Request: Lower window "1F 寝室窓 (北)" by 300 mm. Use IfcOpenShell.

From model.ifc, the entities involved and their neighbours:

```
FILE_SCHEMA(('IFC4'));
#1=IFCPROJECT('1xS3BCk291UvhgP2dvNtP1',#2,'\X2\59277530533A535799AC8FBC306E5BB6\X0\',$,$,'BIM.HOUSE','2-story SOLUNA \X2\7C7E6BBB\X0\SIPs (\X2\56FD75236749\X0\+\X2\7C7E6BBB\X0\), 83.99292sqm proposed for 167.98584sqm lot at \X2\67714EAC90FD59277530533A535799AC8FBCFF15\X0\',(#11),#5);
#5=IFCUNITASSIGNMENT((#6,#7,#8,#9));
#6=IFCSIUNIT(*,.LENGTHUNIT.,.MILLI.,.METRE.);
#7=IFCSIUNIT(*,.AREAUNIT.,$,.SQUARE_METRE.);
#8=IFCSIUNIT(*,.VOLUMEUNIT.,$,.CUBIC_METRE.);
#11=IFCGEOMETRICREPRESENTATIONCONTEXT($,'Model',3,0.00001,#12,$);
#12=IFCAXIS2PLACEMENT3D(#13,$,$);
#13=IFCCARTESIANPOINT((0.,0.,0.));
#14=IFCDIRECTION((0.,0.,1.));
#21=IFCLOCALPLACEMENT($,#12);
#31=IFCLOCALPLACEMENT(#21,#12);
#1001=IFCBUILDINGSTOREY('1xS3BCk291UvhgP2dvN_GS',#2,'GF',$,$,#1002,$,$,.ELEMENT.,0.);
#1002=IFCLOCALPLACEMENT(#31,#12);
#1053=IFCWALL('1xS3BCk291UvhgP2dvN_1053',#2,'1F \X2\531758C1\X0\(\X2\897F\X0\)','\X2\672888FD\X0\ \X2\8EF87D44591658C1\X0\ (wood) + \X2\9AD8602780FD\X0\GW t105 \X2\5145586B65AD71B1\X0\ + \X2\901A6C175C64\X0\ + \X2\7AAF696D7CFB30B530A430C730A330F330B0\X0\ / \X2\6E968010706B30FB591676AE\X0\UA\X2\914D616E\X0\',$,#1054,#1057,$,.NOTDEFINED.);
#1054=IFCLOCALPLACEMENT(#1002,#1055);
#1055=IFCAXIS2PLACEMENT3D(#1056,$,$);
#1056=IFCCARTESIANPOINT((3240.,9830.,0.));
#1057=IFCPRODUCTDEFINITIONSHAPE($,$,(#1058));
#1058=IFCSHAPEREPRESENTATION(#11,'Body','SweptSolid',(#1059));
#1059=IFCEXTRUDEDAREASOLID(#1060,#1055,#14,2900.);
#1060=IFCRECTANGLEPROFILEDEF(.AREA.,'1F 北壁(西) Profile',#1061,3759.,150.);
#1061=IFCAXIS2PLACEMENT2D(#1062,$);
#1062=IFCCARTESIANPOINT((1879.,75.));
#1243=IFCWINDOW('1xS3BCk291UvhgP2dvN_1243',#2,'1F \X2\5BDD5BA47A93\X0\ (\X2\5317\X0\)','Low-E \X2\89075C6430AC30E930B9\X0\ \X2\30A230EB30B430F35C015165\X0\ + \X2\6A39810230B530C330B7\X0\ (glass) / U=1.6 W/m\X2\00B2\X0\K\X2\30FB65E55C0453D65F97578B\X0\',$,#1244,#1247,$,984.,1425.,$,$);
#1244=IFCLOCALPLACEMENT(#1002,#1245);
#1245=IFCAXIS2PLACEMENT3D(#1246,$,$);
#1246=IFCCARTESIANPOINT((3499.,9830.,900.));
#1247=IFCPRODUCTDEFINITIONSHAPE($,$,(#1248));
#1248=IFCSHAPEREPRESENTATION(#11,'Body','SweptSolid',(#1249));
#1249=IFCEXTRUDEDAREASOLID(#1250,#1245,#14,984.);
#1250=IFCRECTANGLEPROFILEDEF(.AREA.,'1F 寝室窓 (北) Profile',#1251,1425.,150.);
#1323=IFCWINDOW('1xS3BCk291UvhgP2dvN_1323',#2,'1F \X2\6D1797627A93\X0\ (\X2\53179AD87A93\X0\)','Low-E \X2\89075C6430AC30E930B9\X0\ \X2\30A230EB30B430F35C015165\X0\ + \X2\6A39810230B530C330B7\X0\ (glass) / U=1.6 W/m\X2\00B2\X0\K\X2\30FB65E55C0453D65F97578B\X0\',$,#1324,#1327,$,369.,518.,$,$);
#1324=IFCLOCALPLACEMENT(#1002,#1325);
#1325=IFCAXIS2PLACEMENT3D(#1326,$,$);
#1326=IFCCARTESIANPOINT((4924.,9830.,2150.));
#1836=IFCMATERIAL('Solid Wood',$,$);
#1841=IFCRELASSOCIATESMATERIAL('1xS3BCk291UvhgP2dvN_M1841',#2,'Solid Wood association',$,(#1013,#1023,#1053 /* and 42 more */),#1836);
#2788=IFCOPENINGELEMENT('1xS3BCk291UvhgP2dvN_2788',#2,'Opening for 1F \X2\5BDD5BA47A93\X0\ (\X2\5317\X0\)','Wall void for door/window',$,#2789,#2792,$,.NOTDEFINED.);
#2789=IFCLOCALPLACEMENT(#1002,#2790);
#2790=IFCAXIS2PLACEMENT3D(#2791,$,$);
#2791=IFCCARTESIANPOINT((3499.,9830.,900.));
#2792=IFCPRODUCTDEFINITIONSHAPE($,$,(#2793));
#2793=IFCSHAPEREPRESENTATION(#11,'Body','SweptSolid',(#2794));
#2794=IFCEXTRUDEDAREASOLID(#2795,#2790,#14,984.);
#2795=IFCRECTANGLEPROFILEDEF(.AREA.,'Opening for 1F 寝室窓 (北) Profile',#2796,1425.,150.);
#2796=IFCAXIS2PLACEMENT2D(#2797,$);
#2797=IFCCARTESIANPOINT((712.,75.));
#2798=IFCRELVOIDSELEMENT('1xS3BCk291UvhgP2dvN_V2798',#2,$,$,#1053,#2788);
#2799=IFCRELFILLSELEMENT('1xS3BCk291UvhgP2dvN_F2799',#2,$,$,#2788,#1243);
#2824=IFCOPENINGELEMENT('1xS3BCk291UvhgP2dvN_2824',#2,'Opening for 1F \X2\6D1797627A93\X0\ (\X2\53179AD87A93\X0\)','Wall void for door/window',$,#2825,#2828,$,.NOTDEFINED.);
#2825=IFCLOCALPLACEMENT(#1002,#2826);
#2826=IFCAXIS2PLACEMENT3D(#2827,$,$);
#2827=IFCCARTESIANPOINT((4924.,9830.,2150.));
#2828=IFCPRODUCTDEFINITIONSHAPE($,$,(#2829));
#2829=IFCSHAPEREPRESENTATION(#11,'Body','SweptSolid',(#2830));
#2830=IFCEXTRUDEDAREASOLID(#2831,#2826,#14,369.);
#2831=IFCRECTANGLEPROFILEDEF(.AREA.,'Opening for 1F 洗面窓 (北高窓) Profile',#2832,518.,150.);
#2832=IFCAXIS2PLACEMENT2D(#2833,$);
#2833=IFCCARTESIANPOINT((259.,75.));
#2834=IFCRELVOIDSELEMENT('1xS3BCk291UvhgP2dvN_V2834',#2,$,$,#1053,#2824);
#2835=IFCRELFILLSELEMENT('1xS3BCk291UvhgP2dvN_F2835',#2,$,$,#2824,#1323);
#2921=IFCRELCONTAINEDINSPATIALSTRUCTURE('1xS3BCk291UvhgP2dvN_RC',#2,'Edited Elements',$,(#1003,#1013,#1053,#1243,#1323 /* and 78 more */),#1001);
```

```python
import numpy as np
import ifcopenshell
import ifcopenshell.api.geometry
import ifcopenshell.util.placement
import ifcopenshell.util.unit

model = ifcopenshell.open("model.ifc")
unit_scale = ifcopenshell.util.unit.calculate_unit_scale(model)

window = model.by_id(1243)
opening = window.FillsVoids[0].RelatingOpeningElement
dz = -0.3 / unit_scale

shift = np.array([0.0, 0.0, dz])
# The window is not placed relative to its opening, so move both.
for product in (opening, window):
    matrix = ifcopenshell.util.placement.get_local_placement(product.ObjectPlacement)
    matrix[:3, 3] += shift
    ifcopenshell.api.geometry.edit_object_placement(model, product=product, matrix=matrix, is_si=False)

print(f"moved by {dz * unit_scale:+.3f} m")

model.write("model_rev.ifc")
```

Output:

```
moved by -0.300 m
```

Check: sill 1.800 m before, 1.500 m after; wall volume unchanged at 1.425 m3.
